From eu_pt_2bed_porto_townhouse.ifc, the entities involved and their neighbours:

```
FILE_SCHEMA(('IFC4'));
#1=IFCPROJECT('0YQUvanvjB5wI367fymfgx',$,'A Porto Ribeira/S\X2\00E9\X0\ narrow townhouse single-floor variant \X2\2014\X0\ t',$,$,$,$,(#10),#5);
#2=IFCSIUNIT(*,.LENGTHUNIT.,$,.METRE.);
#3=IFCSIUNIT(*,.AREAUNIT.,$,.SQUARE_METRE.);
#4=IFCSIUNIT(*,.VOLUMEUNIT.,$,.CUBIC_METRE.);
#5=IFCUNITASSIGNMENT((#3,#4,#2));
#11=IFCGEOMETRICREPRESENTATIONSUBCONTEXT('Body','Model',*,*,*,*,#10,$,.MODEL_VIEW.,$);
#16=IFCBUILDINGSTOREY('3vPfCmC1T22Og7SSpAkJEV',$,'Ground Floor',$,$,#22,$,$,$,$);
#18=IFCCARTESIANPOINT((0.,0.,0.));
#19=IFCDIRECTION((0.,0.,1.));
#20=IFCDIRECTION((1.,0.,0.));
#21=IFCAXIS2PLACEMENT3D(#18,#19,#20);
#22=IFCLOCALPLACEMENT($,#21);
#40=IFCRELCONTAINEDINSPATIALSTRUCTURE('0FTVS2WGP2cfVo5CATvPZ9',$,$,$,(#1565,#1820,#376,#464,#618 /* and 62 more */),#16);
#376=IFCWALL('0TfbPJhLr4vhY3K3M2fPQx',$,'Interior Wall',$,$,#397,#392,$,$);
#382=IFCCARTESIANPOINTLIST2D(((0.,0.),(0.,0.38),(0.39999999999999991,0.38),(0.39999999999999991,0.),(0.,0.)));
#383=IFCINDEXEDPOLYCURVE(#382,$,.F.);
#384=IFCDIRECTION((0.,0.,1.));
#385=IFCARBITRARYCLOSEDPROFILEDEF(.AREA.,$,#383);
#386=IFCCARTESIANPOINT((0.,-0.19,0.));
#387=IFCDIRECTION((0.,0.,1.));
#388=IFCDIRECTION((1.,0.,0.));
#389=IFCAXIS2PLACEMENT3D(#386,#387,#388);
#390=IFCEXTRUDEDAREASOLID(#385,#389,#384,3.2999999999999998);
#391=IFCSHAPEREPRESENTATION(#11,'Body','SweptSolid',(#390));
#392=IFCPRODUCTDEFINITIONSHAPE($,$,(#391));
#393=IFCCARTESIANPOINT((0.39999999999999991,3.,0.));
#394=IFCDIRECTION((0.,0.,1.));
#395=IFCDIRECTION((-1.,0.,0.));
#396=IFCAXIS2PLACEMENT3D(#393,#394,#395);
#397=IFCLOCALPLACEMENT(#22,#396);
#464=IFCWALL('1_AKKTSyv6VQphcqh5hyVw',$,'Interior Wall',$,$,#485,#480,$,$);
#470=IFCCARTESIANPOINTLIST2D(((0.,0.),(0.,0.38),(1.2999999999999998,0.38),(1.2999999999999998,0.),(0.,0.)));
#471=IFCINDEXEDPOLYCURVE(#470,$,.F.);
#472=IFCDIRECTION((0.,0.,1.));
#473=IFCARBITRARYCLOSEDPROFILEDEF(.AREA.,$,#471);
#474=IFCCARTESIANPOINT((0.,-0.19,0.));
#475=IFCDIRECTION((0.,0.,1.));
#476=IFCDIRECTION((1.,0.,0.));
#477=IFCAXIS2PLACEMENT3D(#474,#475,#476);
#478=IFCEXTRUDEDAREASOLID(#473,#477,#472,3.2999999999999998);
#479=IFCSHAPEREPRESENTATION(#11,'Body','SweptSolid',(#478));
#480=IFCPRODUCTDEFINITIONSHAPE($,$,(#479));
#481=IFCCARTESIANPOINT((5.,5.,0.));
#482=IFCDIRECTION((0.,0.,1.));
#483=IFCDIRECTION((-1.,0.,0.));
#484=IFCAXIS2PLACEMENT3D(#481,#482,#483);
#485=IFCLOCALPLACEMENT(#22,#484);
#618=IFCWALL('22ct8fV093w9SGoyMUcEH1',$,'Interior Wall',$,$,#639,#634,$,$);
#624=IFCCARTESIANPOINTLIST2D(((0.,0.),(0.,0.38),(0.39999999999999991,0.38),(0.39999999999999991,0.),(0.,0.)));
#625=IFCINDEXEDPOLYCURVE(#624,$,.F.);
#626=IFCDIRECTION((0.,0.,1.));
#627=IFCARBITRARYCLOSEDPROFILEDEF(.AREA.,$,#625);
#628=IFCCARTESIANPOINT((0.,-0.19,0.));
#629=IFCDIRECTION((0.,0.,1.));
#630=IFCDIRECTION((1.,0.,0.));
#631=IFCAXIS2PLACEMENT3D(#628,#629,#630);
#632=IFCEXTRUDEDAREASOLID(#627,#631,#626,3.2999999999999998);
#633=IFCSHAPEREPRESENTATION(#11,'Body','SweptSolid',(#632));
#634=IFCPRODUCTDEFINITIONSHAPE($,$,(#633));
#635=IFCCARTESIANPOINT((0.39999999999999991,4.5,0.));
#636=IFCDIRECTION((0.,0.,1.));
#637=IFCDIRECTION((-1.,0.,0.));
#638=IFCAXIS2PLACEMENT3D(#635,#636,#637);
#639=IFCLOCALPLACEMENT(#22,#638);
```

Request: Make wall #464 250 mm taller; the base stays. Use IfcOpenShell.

```python
import ifcopenshell
import ifcopenshell.geom
import ifcopenshell.util.representation
import ifcopenshell.util.shape

model = ifcopenshell.open("eu_pt_2bed_porto_townhouse.ifc")
settings = ifcopenshell.geom.settings()


def volume(element):
    """Net volume in cubic metres, openings subtracted."""
    shape = ifcopenshell.geom.create_shape(settings, element)
    return ifcopenshell.util.shape.get_volume(shape.geometry)


wall = model.by_id(464)
before = volume(wall)

body = ifcopenshell.util.representation.get_representation(wall, "Model", "Body")
solid = body.Items[0]
old_height = solid.Depth
solid.Depth += 0.25
after = volume(wall)

print(f"height {old_height:g} -> {solid.Depth:g}, volume {before:.3f} -> {after:.3f} m3")

model.write("eu_pt_2bed_porto_townhouse-out.ifc")
```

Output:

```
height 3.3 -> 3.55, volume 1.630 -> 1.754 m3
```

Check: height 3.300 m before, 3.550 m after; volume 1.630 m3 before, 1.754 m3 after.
